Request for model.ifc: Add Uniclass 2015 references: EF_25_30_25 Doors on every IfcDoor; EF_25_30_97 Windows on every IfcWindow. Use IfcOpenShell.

First a look at what the model holds.

```python
import ifcopenshell

model = ifcopenshell.open("model.ifc")
print(model.schema)
print("classifications:", [c.Name for c in model.by_type("IfcClassification")])
for ifc_class in ("IfcDoor", "IfcRoof", "IfcStair", "IfcWall", "IfcWindow"):
    print(ifc_class, len(model.by_type(ifc_class)))
```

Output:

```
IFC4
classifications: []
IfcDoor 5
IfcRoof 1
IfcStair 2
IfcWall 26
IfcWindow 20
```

```python
import ifcopenshell
import ifcopenshell.api.classification

model = ifcopenshell.open("model.ifc")

system = ifcopenshell.api.classification.add_classification(model, classification="Uniclass 2015")

codes = {
    "IfcDoor": ("EF_25_30_25", "Doors"),
    "IfcWindow": ("EF_25_30_97", "Windows"),
}
for ifc_class, (code, name) in codes.items():
    products = model.by_type(ifc_class)
    ifcopenshell.api.classification.add_reference(
        model, products=products, classification=system, identification=code, name=name
    )
    print(code, len(products))

model.write("model_v2.ifc")
```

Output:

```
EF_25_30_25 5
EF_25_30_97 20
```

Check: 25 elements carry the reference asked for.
